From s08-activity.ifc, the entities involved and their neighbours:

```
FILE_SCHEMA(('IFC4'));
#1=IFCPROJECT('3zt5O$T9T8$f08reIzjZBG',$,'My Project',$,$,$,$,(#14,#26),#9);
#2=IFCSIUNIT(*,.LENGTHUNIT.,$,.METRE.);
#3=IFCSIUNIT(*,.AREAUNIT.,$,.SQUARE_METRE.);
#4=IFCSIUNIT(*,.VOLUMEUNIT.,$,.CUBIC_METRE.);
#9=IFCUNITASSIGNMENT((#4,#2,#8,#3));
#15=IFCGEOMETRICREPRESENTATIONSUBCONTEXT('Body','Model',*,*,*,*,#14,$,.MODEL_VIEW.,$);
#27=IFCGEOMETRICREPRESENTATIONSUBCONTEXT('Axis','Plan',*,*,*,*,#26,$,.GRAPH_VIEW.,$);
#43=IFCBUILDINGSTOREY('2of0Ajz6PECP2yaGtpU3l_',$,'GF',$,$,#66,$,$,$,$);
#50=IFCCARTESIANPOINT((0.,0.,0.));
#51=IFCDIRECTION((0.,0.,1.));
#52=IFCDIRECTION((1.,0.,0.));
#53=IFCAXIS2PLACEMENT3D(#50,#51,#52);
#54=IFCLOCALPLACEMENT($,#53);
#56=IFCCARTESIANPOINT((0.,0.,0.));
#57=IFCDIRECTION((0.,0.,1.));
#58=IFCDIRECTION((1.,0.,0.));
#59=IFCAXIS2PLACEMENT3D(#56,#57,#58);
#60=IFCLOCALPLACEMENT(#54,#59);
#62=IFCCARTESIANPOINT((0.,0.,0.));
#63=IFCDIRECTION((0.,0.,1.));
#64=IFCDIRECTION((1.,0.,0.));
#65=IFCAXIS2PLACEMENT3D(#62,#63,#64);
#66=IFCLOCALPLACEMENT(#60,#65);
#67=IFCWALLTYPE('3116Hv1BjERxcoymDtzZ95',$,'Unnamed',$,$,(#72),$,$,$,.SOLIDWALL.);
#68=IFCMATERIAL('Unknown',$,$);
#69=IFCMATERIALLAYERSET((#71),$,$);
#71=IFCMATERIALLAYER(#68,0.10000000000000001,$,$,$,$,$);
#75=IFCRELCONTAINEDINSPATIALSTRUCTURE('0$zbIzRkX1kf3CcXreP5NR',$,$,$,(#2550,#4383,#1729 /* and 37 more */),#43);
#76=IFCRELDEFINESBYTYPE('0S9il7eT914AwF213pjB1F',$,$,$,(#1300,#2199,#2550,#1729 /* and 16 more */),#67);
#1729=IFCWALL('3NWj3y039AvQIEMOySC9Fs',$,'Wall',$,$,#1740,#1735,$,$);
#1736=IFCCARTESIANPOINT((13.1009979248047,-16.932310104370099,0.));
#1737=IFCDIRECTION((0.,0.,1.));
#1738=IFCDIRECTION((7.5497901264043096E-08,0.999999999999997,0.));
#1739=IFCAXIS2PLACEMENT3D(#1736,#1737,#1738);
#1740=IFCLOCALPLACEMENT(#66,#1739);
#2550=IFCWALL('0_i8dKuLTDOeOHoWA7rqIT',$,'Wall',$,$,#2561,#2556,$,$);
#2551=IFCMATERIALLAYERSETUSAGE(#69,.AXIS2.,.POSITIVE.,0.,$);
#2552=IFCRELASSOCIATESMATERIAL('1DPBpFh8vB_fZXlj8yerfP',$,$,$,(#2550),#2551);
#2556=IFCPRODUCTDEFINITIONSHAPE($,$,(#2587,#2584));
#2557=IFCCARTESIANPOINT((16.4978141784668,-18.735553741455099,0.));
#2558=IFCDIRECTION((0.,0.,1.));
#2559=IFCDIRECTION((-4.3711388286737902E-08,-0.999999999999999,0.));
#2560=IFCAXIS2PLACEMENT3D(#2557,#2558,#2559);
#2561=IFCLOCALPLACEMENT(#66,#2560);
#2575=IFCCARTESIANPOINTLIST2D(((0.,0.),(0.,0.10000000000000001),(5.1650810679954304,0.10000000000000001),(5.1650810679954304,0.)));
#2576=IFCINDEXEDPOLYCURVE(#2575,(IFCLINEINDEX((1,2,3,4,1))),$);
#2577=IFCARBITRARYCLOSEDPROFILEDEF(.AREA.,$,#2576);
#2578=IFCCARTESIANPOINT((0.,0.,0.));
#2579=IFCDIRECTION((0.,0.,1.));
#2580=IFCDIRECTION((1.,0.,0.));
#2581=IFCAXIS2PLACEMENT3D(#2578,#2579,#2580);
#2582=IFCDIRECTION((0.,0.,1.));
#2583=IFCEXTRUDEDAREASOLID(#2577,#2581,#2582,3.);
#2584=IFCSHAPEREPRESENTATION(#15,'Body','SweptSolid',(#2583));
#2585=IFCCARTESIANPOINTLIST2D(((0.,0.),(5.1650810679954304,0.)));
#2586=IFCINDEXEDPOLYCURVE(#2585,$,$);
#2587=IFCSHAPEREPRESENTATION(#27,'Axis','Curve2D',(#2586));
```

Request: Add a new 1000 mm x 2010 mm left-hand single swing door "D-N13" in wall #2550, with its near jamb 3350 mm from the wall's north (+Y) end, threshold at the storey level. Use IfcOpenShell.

```python
import numpy as np
import ifcopenshell
import ifcopenshell.api.feature
import ifcopenshell.api.geometry
import ifcopenshell.api.root
import ifcopenshell.api.spatial
import ifcopenshell.geom
import ifcopenshell.util.element
import ifcopenshell.util.placement
import ifcopenshell.util.representation
import ifcopenshell.util.shape
import ifcopenshell.util.unit

model = ifcopenshell.open("s08-activity.ifc")
unit_scale = ifcopenshell.util.unit.calculate_unit_scale(model)
settings = ifcopenshell.geom.settings()


def volume(element):
    """Net volume in cubic metres, openings subtracted."""
    shape = ifcopenshell.geom.create_shape(settings, element)
    return ifcopenshell.util.shape.get_volume(shape.geometry)


wall = model.by_guid("0_i8dKuLTDOeOHoWA7rqIT")
storey = ifcopenshell.util.element.get_container(wall, ifc_class="IfcBuildingStorey")
context = ifcopenshell.util.representation.get_context(model, "Model", "Body", "MODEL_VIEW")
before = volume(wall)

width, height, from_end, sill = 1, 2.01, 3.35, 0.0  # metres

# The wall runs along its own X axis, and the end named is its -X end.
wall_shape = ifcopenshell.geom.create_shape(settings, wall)
x, y, z = ifcopenshell.util.shape.get_vertices(wall_shape.geometry).T
start = x.min() + from_end
face, thickness = float(y.min()), float(y.max() - y.min())
wall_matrix = ifcopenshell.util.placement.get_local_placement(wall.ObjectPlacement)
level = ifcopenshell.util.placement.get_local_placement(storey.ObjectPlacement)[2, 3]


def in_wall(x, y):
    """Placement at x, y metres in the wall's axes, at sill height."""
    matrix = wall_matrix.copy()
    matrix[:, 3] = wall_matrix @ np.array([x / unit_scale, y / unit_scale, 0.0, 1.0])
    matrix[2, 3] = level + sill / unit_scale
    return matrix


# Opening: a box that overshoots both wall faces by 50 mm.
opening = ifcopenshell.api.root.create_entity(model, ifc_class="IfcOpeningElement", predefined_type="OPENING")
box = ifcopenshell.api.geometry.add_wall_representation(
    model, context=context, length=width, height=height, thickness=thickness + 0.1
)
ifcopenshell.api.geometry.assign_representation(model, product=opening, representation=box)
ifcopenshell.api.geometry.edit_object_placement(model, product=opening, matrix=in_wall(start, face - 0.05), is_si=False)
ifcopenshell.api.feature.add_feature(model, feature=opening, element=wall)

door = ifcopenshell.api.root.create_entity(model, ifc_class="IfcDoor", name="D-N13", predefined_type="DOOR")
door.OverallWidth, door.OverallHeight = width / unit_scale, height / unit_scale
door.OperationType = "SINGLE_SWING_LEFT"
body = ifcopenshell.api.geometry.add_door_representation(
    model,
    context=context,
    overall_width=door.OverallWidth,
    overall_height=door.OverallHeight,
    operation_type="SINGLE_SWING_LEFT",
    lining_properties={"LiningDepth": thickness / unit_scale, "ThresholdDepth": thickness / unit_scale},
)
ifcopenshell.api.geometry.assign_representation(model, product=door, representation=body)
ifcopenshell.api.spatial.assign_container(model, products=[door], relating_structure=storey)
ifcopenshell.api.feature.add_filling(model, opening=opening, element=door)

# The lining spans the wall, so the door starts at the wall face.
ifcopenshell.api.geometry.edit_object_placement(model, product=door, matrix=in_wall(start, face), is_si=False)

after = volume(wall)

print(f"wall volume {before:.3f} -> {after:.3f} m3")

model.write("s08-activity_updated.ifc")
```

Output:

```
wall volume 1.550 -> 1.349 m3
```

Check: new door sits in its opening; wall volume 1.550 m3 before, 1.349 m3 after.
